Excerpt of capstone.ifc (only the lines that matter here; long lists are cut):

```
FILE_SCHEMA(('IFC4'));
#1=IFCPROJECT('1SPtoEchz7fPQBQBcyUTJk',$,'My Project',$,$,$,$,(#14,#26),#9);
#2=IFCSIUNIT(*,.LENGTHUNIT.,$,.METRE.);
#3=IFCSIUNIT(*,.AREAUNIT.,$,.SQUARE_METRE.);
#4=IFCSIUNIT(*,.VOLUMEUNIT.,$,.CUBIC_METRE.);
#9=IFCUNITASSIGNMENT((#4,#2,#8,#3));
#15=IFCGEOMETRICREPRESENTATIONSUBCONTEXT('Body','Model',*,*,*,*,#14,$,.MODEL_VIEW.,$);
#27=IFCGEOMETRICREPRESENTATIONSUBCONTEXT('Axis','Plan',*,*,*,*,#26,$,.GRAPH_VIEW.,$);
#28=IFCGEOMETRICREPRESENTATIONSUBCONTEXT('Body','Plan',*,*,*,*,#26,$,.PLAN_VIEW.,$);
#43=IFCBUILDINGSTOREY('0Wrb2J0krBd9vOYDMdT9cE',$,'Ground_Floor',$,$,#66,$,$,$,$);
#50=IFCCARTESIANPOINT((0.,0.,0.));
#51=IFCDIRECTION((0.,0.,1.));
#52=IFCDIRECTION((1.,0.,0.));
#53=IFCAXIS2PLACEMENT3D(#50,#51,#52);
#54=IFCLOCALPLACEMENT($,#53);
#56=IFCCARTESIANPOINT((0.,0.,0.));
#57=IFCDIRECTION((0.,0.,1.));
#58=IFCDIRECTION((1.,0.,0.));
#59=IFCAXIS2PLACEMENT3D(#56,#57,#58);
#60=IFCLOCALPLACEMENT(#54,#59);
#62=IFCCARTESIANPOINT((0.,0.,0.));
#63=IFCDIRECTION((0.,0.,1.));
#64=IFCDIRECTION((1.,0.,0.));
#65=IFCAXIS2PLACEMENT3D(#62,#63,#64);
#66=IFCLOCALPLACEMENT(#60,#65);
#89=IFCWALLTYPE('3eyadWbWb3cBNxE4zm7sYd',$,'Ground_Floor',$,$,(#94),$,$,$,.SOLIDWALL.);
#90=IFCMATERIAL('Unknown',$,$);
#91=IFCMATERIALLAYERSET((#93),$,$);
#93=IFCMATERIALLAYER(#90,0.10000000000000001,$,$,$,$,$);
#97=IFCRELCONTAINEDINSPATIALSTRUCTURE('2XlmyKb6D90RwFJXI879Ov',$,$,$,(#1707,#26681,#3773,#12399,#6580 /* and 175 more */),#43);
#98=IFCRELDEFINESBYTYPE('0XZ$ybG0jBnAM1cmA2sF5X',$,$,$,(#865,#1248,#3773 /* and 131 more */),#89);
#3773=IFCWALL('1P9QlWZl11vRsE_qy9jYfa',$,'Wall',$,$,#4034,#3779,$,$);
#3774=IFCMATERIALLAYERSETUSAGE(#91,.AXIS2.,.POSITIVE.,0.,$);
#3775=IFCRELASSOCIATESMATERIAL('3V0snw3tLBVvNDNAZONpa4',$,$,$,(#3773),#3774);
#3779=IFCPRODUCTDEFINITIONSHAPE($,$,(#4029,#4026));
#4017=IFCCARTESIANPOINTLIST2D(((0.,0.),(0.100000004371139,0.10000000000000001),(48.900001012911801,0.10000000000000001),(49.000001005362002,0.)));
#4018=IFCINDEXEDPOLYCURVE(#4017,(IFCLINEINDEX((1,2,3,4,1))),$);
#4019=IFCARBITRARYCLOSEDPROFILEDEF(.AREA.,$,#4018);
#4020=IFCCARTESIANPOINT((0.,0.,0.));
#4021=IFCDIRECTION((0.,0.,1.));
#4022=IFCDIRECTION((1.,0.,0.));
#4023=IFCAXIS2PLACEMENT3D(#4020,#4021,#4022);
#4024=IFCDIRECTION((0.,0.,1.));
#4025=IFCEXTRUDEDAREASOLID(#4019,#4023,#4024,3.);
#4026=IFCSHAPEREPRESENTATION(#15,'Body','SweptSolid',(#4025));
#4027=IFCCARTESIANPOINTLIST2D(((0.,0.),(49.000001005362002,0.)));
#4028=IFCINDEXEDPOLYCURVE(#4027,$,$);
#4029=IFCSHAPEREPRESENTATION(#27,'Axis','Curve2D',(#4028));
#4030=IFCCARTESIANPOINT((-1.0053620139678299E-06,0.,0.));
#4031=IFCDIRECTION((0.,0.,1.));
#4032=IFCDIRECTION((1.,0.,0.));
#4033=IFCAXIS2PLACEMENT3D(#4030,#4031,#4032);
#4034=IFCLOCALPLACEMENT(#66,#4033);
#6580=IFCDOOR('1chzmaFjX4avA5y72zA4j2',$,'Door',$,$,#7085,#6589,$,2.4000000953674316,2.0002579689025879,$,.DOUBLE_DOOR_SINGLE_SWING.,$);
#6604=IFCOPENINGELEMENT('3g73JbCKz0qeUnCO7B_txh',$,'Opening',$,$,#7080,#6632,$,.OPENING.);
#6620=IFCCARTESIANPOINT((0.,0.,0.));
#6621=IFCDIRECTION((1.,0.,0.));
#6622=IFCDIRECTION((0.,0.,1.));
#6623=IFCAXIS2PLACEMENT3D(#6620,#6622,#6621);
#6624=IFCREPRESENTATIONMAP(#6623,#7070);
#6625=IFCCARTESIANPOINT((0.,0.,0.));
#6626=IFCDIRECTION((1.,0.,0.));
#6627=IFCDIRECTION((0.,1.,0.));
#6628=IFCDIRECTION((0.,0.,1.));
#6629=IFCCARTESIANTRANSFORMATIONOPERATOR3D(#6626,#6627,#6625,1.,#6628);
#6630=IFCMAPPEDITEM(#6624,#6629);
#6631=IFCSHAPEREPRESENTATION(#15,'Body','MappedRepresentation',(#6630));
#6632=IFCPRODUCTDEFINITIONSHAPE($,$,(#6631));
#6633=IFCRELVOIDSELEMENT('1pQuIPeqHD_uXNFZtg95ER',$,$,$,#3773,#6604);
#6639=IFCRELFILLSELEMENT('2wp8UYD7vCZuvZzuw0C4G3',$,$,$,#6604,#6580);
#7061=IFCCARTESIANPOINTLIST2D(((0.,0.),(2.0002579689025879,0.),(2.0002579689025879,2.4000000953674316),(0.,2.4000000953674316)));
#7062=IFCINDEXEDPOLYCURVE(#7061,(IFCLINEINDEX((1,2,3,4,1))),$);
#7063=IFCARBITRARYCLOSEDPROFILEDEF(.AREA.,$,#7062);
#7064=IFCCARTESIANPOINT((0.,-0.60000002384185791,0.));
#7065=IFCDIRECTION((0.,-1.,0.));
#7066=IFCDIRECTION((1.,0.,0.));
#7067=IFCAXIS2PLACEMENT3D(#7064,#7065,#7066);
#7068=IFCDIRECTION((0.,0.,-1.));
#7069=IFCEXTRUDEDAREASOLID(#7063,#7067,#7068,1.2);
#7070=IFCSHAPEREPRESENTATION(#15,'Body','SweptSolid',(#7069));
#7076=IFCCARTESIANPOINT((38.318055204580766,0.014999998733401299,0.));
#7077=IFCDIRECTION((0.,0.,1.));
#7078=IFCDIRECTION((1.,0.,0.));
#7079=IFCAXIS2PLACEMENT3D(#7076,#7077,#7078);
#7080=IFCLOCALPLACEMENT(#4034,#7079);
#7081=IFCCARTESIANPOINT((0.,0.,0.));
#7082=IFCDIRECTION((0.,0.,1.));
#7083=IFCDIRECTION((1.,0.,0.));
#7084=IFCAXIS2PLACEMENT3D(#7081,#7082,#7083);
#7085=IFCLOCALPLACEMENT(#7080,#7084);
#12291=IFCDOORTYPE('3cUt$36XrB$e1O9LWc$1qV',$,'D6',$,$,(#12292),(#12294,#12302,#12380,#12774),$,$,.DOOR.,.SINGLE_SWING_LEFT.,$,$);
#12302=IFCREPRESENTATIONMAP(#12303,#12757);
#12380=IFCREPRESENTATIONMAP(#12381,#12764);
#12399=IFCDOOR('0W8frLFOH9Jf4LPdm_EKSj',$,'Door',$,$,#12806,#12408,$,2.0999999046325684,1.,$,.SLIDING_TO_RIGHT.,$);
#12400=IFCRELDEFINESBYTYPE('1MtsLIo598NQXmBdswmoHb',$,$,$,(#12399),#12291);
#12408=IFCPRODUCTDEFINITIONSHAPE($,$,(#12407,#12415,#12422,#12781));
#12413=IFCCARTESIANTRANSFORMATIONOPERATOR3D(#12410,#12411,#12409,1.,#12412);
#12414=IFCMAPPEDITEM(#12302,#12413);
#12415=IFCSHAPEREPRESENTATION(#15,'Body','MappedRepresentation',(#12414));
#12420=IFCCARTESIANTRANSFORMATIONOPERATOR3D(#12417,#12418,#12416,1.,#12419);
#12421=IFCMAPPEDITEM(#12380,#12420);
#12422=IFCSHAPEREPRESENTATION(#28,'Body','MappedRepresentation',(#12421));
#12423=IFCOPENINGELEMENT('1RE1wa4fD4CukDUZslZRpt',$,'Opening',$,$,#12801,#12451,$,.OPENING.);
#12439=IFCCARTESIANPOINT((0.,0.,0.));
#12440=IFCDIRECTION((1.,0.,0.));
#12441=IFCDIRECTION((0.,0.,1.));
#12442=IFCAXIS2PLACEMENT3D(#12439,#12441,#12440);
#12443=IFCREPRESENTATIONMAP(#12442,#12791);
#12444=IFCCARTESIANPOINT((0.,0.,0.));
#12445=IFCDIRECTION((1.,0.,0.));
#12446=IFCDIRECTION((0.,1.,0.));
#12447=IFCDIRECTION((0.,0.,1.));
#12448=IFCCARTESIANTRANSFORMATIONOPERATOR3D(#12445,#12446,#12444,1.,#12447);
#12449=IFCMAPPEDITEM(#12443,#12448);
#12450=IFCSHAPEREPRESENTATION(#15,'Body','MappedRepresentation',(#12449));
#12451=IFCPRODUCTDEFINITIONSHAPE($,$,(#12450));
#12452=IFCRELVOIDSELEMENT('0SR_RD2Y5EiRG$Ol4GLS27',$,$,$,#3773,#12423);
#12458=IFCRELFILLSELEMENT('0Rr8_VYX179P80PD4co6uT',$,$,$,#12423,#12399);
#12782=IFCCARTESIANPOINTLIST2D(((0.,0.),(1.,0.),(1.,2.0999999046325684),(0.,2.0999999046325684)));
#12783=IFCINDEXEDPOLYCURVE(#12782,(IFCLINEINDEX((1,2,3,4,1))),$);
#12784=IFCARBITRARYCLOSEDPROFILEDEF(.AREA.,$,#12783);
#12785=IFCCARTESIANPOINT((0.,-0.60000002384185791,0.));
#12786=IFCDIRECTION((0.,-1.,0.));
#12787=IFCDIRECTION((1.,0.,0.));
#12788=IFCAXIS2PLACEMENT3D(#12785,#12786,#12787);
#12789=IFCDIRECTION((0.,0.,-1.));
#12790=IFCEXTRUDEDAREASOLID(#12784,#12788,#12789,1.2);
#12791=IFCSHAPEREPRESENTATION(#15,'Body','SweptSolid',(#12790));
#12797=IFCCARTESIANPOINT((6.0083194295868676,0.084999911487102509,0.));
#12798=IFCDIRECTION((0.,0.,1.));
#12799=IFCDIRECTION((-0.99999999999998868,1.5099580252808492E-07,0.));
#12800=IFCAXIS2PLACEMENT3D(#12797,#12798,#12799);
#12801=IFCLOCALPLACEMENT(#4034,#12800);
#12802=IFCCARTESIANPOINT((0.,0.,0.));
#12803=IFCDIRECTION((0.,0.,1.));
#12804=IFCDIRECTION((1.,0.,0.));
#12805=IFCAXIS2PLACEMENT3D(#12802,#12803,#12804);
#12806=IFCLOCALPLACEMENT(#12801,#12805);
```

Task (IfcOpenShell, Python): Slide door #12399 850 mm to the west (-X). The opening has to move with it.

```python
import ifcopenshell
import ifcopenshell.api.geometry
import ifcopenshell.util.placement
import ifcopenshell.util.unit

model = ifcopenshell.open("capstone.ifc")
unit_scale = ifcopenshell.util.unit.calculate_unit_scale(model)

door = model.by_guid("0W8frLFOH9Jf4LPdm_EKSj")
opening = door.FillsVoids[0].RelatingOpeningElement
wall = opening.VoidsElements[0].RelatingBuildingElement

wall_matrix = ifcopenshell.util.placement.get_local_placement(wall.ObjectPlacement)
shift = wall_matrix[:3, 0] * -0.85 / unit_scale
before = ifcopenshell.util.placement.get_local_placement(door.ObjectPlacement)[:3, 3].copy()

# The door is placed relative to its opening, so it follows when the opening moves.
matrix = ifcopenshell.util.placement.get_local_placement(opening.ObjectPlacement)
matrix[:3, 3] += shift
ifcopenshell.api.geometry.edit_object_placement(
    model, product=opening, matrix=matrix, is_si=False, should_transform_children=True
)

after = ifcopenshell.util.placement.get_local_placement(door.ObjectPlacement)[:3, 3]
print("door moved by", (after - before).round(3) + 0.0)

model.write("capstone-out.ifc")
```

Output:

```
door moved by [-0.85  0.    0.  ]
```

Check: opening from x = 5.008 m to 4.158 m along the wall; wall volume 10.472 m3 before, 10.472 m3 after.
